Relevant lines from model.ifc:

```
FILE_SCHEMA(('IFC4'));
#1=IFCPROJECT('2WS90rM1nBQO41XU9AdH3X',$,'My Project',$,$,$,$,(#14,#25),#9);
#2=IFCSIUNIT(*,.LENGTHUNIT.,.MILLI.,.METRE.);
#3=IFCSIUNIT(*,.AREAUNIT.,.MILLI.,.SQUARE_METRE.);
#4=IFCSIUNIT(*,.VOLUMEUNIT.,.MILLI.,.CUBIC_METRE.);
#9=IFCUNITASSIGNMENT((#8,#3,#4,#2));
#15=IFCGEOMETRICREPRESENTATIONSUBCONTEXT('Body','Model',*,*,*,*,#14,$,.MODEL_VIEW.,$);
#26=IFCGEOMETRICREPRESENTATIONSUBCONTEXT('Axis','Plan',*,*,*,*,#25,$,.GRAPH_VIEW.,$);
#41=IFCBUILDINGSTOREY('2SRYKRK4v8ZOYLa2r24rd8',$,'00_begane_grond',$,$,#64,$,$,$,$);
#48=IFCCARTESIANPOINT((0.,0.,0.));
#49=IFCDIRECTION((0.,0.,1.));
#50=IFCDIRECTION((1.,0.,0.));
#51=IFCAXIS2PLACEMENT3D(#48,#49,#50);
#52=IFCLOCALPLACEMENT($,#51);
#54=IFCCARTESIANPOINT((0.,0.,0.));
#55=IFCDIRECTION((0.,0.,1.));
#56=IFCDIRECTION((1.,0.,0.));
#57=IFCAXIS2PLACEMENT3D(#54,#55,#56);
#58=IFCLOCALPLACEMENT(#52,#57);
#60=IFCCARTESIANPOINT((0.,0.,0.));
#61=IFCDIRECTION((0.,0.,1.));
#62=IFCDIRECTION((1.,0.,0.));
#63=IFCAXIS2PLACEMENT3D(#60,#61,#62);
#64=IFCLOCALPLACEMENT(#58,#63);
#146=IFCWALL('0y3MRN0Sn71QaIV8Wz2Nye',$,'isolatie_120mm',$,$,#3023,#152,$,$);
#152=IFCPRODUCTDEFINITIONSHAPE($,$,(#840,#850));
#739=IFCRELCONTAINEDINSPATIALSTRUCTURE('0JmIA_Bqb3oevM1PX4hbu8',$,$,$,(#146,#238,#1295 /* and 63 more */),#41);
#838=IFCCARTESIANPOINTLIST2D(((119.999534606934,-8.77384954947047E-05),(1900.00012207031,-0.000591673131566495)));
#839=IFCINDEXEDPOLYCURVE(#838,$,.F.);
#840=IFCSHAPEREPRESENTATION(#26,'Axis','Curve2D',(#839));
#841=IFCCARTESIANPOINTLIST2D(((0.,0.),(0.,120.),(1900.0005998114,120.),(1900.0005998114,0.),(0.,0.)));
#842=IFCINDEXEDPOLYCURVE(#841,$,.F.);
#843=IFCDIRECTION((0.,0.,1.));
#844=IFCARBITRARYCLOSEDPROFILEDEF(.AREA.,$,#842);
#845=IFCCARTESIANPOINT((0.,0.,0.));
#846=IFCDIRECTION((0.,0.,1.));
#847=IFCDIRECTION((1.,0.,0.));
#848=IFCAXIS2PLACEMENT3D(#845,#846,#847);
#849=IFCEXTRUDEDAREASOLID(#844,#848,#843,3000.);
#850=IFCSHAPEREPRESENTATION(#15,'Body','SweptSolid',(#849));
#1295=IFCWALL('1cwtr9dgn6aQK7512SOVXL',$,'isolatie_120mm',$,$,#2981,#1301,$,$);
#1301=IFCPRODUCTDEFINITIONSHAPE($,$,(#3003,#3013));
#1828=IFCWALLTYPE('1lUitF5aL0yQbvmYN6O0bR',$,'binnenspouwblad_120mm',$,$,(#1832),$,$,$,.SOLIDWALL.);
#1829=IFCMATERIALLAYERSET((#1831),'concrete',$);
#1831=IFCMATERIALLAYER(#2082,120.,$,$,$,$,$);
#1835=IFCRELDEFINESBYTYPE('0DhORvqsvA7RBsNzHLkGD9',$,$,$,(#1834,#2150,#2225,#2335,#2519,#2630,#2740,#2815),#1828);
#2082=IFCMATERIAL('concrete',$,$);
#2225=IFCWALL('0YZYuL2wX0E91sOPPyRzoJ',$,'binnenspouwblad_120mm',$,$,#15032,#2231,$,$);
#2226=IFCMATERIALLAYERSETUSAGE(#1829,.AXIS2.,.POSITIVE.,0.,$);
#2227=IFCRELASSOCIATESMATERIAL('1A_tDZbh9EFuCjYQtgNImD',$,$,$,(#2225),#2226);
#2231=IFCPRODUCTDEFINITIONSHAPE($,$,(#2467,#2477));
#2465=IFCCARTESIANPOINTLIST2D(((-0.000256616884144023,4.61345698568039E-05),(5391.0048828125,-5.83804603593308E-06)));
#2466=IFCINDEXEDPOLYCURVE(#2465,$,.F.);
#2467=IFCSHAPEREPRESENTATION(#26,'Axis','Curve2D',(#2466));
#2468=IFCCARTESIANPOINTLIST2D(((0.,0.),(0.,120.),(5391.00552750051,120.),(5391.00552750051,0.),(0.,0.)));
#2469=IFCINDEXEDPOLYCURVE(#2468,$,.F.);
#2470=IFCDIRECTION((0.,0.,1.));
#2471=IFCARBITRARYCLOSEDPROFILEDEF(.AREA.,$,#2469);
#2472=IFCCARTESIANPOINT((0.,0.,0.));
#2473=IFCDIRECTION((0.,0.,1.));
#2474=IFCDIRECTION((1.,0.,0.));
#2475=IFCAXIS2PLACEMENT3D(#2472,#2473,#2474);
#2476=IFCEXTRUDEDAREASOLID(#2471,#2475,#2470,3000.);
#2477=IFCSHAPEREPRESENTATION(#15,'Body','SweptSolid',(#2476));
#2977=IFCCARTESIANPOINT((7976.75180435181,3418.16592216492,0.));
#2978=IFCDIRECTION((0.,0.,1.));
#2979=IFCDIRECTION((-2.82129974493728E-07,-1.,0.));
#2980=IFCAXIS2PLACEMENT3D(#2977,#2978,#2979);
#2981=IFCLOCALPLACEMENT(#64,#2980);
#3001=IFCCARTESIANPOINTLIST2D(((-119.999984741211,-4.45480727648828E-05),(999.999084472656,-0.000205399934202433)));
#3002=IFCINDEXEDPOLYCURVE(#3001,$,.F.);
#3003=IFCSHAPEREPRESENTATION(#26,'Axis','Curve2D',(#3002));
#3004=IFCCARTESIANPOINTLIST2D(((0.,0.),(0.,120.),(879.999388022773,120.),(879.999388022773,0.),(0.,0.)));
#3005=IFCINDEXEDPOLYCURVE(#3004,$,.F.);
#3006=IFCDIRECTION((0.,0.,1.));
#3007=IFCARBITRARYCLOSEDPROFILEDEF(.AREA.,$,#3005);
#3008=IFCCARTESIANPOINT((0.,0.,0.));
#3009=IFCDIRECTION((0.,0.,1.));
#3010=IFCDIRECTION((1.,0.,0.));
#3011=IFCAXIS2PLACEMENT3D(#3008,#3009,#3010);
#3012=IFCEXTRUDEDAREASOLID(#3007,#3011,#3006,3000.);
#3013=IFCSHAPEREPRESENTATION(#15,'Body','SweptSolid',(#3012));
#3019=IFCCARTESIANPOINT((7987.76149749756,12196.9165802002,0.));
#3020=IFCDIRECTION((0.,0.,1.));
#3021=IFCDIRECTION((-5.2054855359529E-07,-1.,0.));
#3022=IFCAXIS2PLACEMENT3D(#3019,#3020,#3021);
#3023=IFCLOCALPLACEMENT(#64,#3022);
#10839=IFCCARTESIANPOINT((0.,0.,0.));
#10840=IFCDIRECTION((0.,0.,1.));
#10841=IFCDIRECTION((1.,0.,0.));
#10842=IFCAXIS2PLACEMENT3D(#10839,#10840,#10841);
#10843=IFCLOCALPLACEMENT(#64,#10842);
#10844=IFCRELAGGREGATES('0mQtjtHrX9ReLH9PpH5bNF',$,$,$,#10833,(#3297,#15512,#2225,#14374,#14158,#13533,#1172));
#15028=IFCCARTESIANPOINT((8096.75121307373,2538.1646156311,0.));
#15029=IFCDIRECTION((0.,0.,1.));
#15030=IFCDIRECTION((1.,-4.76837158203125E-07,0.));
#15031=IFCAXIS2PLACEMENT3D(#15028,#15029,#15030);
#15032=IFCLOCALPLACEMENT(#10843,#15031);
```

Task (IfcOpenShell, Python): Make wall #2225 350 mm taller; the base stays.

```python
import ifcopenshell
import ifcopenshell.geom
import ifcopenshell.util.representation
import ifcopenshell.util.shape

model = ifcopenshell.open("model.ifc")
settings = ifcopenshell.geom.settings()


def volume(element):
    """Net volume in cubic metres, openings subtracted."""
    shape = ifcopenshell.geom.create_shape(settings, element)
    return ifcopenshell.util.shape.get_volume(shape.geometry)


wall = model.by_guid("0YZYuL2wX0E91sOPPyRzoJ")
before = volume(wall)

body = ifcopenshell.util.representation.get_representation(wall, "Model", "Body")
solid = body.Items[0]
old_height = solid.Depth
solid.Depth += 350.0
after = volume(wall)

print(f"height {old_height:g} -> {solid.Depth:g}, volume {before:.3f} -> {after:.3f} m3")

model.write("model_v2.ifc")
```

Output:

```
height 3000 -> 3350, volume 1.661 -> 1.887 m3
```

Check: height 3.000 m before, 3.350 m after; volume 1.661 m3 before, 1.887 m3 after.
